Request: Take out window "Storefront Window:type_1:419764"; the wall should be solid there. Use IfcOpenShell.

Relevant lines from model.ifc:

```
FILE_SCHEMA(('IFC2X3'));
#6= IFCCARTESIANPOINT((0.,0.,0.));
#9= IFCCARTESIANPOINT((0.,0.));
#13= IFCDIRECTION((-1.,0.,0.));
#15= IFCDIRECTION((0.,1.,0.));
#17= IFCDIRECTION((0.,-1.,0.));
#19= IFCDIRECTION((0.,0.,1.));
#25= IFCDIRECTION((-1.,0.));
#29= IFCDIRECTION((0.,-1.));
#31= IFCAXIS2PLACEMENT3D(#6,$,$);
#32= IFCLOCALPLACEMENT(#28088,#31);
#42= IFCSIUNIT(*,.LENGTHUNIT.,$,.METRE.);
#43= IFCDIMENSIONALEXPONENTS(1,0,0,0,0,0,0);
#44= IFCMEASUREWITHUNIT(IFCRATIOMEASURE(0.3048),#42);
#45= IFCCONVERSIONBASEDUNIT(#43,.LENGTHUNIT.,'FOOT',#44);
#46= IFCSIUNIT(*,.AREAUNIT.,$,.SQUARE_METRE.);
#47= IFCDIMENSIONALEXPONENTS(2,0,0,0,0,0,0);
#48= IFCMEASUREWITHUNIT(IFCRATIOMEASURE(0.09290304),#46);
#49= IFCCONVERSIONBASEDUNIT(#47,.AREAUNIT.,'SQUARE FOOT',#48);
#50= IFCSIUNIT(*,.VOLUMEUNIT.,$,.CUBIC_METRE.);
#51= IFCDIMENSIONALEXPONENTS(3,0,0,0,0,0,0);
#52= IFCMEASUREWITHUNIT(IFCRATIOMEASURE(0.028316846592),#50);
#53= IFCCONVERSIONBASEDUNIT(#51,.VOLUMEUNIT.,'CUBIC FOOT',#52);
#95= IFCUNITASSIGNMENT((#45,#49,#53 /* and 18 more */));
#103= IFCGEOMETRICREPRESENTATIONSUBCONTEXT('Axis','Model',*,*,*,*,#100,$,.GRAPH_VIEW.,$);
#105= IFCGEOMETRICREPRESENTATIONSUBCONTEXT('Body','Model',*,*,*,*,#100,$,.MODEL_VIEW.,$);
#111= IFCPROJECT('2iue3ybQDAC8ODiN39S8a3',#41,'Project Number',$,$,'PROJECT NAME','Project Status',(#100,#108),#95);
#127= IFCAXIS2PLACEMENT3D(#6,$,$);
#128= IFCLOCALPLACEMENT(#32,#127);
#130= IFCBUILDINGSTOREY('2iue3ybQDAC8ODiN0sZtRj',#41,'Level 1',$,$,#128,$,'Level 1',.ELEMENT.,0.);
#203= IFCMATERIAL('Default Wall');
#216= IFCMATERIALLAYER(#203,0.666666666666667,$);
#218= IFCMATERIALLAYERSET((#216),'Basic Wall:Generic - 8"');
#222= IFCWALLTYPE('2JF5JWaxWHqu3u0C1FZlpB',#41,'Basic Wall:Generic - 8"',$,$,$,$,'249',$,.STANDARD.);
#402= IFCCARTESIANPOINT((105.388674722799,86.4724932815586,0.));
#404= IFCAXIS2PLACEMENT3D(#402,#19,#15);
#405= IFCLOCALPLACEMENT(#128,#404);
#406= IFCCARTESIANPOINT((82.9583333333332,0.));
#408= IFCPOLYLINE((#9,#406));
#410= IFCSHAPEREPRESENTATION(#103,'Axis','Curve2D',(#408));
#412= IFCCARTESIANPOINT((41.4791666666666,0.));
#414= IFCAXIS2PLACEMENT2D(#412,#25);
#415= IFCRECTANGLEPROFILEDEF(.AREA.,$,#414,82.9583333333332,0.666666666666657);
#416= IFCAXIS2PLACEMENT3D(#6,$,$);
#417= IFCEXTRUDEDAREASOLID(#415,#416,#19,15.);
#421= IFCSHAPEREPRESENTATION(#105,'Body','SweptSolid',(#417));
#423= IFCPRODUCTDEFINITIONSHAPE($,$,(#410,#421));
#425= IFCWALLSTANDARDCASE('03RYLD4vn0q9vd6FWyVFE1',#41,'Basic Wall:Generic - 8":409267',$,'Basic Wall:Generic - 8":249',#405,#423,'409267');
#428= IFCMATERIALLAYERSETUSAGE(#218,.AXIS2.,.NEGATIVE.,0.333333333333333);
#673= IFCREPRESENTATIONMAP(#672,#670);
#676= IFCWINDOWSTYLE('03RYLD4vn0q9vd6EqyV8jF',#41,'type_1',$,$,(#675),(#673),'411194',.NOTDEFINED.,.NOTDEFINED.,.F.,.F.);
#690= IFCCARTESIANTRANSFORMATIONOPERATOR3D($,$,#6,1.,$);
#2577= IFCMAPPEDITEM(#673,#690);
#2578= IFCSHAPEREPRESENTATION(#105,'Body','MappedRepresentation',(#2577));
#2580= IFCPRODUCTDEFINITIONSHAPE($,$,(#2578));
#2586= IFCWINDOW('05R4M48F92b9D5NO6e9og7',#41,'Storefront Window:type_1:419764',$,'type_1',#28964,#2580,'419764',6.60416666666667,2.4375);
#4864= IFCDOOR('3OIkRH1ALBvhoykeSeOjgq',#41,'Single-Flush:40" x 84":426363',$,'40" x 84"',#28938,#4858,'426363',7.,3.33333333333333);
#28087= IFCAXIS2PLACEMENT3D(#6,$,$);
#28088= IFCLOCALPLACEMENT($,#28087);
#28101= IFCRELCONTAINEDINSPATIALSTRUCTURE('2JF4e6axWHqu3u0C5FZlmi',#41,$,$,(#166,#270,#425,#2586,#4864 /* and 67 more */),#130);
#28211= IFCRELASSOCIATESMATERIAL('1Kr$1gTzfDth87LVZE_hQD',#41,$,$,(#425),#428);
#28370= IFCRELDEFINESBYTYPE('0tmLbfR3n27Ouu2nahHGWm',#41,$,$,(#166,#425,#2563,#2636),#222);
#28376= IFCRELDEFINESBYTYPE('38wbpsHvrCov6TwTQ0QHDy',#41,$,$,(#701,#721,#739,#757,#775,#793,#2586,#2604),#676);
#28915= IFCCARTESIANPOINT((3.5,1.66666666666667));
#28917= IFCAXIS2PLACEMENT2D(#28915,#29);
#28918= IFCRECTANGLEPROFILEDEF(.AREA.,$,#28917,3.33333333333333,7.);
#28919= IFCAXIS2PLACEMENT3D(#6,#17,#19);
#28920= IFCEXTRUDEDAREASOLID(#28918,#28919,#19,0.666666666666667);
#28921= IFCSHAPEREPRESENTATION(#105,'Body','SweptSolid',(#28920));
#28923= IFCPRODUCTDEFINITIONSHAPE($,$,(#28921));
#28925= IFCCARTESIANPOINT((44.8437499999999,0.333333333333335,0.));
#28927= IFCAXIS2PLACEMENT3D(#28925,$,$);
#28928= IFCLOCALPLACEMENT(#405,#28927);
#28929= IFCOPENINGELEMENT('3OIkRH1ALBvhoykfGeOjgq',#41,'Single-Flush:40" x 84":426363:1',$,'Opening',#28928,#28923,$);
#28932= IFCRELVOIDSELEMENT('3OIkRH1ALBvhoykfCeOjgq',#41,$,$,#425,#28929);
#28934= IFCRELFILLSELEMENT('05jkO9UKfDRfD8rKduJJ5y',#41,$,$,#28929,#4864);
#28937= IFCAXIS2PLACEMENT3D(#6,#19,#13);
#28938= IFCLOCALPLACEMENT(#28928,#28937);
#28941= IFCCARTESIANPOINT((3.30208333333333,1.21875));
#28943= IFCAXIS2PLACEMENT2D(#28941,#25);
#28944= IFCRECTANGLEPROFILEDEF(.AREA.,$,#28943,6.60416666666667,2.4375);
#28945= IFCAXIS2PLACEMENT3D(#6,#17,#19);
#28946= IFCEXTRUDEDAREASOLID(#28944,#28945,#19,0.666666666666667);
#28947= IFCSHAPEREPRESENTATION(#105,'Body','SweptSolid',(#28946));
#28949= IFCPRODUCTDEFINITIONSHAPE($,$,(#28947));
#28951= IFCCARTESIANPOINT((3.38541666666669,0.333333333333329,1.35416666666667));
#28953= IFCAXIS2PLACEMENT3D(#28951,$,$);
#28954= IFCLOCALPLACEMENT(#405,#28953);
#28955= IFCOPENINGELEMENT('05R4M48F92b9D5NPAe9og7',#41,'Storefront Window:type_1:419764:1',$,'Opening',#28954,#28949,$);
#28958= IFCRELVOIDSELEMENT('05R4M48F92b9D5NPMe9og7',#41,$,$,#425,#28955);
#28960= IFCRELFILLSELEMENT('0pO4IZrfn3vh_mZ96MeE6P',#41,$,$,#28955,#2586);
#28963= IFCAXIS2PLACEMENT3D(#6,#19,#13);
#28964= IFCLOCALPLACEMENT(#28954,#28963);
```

```python
import ifcopenshell
import ifcopenshell.api.feature
import ifcopenshell.api.root
import ifcopenshell.geom
import ifcopenshell.util.shape

model = ifcopenshell.open("model.ifc")
settings = ifcopenshell.geom.settings()


def volume(element):
    """Net volume in cubic metres, openings subtracted."""
    shape = ifcopenshell.geom.create_shape(settings, element)
    return ifcopenshell.util.shape.get_volume(shape.geometry)


window = model.by_guid("05R4M48F92b9D5NO6e9og7")
opening = window.FillsVoids[0].RelatingOpeningElement
wall = opening.VoidsElements[0].RelatingBuildingElement
before = volume(wall)

ifcopenshell.api.root.remove_product(model, product=window)
ifcopenshell.api.feature.remove_feature(model, feature=opening)

after = volume(wall)

print(f"wall volume {before:.3f} -> {after:.3f} m3")

model.write("model_updated.ifc")
```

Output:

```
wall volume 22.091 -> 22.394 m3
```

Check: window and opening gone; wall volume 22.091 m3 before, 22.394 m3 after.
